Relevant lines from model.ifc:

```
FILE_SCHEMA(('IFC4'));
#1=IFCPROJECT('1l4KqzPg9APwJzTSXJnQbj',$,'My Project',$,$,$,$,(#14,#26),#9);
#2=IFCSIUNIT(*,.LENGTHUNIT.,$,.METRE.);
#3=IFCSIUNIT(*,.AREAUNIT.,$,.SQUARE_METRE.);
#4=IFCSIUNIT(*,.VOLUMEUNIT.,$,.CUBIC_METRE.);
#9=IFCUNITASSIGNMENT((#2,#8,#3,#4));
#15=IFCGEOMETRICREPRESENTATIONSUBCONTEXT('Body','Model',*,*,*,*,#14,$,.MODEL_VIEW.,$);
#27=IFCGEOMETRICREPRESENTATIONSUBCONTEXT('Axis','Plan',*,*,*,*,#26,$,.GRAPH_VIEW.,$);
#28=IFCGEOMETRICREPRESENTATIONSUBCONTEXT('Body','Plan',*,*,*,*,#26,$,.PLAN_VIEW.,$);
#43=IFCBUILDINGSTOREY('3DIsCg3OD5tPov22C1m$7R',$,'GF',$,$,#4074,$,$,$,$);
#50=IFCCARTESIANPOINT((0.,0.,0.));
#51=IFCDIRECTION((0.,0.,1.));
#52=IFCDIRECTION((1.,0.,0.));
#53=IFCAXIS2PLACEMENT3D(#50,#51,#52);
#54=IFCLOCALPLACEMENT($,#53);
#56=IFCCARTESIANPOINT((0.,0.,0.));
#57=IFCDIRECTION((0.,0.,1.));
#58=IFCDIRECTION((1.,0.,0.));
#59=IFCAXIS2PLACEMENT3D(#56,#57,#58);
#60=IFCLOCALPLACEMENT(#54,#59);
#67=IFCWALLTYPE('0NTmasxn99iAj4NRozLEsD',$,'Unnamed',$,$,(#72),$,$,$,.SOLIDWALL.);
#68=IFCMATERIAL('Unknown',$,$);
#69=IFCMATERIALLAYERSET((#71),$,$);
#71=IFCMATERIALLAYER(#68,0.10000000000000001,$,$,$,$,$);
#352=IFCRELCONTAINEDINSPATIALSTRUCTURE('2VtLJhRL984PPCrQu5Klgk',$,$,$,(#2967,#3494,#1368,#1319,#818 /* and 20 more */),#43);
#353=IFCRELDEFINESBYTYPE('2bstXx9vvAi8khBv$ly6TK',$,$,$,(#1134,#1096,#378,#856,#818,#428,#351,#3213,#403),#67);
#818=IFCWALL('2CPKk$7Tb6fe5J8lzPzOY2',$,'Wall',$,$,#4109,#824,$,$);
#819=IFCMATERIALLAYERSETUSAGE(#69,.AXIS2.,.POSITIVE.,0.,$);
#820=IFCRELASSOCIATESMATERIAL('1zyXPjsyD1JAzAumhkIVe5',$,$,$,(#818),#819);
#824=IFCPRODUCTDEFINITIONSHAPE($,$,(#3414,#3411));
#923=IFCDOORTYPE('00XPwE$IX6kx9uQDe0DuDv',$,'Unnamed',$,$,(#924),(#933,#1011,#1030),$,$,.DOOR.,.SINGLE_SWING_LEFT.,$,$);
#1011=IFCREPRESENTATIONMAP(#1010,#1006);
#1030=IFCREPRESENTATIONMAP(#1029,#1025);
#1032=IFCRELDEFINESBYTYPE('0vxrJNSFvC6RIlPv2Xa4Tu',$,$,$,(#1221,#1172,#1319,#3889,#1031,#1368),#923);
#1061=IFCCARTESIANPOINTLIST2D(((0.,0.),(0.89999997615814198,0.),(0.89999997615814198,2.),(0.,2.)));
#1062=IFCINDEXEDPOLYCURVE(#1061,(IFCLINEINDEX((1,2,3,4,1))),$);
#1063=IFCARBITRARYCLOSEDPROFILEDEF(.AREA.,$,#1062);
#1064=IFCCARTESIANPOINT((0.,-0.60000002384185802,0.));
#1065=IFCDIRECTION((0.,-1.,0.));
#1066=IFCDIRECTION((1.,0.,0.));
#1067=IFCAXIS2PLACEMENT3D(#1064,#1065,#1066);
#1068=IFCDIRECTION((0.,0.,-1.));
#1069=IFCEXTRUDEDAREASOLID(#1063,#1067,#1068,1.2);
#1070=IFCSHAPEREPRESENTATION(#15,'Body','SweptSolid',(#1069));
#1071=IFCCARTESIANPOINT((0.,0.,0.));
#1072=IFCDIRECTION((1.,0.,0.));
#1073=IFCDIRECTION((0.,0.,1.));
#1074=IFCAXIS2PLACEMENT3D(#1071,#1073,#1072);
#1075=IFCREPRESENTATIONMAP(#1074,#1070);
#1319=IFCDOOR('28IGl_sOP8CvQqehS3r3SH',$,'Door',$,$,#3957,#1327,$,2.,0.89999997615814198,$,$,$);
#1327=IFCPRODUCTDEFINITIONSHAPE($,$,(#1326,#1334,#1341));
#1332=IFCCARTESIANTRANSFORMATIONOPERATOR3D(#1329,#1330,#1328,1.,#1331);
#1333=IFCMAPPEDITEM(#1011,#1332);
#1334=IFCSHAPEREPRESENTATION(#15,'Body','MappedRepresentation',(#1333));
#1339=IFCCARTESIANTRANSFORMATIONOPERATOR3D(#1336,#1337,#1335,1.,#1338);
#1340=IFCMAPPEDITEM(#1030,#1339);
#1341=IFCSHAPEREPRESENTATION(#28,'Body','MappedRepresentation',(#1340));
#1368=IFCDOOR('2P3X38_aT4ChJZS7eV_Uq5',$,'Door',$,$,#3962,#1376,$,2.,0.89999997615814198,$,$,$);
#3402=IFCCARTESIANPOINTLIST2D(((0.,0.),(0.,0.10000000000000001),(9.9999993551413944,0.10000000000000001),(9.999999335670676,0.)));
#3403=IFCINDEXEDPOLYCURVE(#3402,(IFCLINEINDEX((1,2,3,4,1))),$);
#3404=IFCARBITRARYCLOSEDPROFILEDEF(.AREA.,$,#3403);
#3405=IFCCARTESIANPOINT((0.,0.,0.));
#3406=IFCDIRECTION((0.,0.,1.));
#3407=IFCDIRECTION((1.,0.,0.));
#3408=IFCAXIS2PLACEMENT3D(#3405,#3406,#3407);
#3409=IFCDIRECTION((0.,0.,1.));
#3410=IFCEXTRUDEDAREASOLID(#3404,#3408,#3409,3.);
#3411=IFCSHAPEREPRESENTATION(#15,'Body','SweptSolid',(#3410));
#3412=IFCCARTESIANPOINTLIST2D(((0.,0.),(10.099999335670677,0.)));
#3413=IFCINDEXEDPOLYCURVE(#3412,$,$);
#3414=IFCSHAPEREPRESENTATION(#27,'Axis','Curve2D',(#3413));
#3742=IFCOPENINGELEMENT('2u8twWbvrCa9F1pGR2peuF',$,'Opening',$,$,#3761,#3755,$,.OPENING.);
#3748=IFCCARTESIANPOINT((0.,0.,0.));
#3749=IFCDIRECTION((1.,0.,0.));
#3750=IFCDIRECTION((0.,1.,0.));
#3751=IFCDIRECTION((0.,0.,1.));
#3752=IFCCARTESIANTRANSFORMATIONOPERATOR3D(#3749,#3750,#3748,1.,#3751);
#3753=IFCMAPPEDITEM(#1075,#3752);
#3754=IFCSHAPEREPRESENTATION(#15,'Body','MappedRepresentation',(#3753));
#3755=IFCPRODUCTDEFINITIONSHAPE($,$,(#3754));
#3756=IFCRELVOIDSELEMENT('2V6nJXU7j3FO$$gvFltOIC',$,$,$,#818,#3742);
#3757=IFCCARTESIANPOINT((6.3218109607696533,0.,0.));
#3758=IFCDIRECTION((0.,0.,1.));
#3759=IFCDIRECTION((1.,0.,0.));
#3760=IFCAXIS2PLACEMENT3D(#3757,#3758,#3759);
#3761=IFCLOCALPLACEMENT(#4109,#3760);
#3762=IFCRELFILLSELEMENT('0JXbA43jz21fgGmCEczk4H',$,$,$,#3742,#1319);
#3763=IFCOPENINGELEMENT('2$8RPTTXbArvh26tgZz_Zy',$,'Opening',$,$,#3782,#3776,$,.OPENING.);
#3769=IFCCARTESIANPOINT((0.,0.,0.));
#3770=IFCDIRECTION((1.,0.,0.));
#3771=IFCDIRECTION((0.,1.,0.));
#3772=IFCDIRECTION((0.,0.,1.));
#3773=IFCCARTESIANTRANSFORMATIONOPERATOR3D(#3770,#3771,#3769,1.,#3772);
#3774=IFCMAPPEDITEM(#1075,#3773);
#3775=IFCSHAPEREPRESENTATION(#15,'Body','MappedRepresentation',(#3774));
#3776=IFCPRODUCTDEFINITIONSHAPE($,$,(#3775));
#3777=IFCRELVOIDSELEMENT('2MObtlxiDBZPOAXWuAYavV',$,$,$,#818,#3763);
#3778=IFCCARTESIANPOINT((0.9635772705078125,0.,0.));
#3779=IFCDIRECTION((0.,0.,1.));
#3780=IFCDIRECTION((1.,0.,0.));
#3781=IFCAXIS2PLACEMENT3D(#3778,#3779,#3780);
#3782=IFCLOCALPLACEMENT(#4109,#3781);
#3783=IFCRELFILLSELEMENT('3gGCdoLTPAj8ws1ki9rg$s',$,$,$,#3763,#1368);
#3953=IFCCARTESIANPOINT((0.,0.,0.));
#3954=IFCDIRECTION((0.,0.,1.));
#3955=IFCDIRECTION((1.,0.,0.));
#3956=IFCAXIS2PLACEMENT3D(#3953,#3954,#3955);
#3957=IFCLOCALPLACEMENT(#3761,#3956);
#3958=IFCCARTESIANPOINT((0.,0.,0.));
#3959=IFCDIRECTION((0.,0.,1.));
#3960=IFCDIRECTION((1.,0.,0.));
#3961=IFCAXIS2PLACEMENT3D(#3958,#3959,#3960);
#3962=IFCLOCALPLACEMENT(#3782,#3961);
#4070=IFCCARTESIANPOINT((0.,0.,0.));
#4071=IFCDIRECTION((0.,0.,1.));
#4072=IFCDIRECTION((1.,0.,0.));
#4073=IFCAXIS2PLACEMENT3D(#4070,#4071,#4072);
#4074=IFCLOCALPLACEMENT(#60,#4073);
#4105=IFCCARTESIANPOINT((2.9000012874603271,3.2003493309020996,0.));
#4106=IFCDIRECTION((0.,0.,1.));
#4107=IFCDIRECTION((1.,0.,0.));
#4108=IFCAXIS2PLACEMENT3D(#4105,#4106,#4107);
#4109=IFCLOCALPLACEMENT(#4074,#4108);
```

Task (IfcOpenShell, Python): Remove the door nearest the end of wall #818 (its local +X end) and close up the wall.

```python
import ifcopenshell
import ifcopenshell.api.feature
import ifcopenshell.api.root
import ifcopenshell.geom
import ifcopenshell.util.shape

model = ifcopenshell.open("model.ifc")
settings = ifcopenshell.geom.settings()


def volume(element):
    """Net volume in cubic metres, openings subtracted."""
    shape = ifcopenshell.geom.create_shape(settings, element)
    return ifcopenshell.util.shape.get_volume(shape.geometry)


door = model.by_id(1319)
opening = door.FillsVoids[0].RelatingOpeningElement
wall = opening.VoidsElements[0].RelatingBuildingElement
before = volume(wall)

ifcopenshell.api.root.remove_product(model, product=door)
ifcopenshell.api.feature.remove_feature(model, feature=opening)

after = volume(wall)

print(f"wall volume {before:.3f} -> {after:.3f} m3")

model.write("model_v2.ifc")
```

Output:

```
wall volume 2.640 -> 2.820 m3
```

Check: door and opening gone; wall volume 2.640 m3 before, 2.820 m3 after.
